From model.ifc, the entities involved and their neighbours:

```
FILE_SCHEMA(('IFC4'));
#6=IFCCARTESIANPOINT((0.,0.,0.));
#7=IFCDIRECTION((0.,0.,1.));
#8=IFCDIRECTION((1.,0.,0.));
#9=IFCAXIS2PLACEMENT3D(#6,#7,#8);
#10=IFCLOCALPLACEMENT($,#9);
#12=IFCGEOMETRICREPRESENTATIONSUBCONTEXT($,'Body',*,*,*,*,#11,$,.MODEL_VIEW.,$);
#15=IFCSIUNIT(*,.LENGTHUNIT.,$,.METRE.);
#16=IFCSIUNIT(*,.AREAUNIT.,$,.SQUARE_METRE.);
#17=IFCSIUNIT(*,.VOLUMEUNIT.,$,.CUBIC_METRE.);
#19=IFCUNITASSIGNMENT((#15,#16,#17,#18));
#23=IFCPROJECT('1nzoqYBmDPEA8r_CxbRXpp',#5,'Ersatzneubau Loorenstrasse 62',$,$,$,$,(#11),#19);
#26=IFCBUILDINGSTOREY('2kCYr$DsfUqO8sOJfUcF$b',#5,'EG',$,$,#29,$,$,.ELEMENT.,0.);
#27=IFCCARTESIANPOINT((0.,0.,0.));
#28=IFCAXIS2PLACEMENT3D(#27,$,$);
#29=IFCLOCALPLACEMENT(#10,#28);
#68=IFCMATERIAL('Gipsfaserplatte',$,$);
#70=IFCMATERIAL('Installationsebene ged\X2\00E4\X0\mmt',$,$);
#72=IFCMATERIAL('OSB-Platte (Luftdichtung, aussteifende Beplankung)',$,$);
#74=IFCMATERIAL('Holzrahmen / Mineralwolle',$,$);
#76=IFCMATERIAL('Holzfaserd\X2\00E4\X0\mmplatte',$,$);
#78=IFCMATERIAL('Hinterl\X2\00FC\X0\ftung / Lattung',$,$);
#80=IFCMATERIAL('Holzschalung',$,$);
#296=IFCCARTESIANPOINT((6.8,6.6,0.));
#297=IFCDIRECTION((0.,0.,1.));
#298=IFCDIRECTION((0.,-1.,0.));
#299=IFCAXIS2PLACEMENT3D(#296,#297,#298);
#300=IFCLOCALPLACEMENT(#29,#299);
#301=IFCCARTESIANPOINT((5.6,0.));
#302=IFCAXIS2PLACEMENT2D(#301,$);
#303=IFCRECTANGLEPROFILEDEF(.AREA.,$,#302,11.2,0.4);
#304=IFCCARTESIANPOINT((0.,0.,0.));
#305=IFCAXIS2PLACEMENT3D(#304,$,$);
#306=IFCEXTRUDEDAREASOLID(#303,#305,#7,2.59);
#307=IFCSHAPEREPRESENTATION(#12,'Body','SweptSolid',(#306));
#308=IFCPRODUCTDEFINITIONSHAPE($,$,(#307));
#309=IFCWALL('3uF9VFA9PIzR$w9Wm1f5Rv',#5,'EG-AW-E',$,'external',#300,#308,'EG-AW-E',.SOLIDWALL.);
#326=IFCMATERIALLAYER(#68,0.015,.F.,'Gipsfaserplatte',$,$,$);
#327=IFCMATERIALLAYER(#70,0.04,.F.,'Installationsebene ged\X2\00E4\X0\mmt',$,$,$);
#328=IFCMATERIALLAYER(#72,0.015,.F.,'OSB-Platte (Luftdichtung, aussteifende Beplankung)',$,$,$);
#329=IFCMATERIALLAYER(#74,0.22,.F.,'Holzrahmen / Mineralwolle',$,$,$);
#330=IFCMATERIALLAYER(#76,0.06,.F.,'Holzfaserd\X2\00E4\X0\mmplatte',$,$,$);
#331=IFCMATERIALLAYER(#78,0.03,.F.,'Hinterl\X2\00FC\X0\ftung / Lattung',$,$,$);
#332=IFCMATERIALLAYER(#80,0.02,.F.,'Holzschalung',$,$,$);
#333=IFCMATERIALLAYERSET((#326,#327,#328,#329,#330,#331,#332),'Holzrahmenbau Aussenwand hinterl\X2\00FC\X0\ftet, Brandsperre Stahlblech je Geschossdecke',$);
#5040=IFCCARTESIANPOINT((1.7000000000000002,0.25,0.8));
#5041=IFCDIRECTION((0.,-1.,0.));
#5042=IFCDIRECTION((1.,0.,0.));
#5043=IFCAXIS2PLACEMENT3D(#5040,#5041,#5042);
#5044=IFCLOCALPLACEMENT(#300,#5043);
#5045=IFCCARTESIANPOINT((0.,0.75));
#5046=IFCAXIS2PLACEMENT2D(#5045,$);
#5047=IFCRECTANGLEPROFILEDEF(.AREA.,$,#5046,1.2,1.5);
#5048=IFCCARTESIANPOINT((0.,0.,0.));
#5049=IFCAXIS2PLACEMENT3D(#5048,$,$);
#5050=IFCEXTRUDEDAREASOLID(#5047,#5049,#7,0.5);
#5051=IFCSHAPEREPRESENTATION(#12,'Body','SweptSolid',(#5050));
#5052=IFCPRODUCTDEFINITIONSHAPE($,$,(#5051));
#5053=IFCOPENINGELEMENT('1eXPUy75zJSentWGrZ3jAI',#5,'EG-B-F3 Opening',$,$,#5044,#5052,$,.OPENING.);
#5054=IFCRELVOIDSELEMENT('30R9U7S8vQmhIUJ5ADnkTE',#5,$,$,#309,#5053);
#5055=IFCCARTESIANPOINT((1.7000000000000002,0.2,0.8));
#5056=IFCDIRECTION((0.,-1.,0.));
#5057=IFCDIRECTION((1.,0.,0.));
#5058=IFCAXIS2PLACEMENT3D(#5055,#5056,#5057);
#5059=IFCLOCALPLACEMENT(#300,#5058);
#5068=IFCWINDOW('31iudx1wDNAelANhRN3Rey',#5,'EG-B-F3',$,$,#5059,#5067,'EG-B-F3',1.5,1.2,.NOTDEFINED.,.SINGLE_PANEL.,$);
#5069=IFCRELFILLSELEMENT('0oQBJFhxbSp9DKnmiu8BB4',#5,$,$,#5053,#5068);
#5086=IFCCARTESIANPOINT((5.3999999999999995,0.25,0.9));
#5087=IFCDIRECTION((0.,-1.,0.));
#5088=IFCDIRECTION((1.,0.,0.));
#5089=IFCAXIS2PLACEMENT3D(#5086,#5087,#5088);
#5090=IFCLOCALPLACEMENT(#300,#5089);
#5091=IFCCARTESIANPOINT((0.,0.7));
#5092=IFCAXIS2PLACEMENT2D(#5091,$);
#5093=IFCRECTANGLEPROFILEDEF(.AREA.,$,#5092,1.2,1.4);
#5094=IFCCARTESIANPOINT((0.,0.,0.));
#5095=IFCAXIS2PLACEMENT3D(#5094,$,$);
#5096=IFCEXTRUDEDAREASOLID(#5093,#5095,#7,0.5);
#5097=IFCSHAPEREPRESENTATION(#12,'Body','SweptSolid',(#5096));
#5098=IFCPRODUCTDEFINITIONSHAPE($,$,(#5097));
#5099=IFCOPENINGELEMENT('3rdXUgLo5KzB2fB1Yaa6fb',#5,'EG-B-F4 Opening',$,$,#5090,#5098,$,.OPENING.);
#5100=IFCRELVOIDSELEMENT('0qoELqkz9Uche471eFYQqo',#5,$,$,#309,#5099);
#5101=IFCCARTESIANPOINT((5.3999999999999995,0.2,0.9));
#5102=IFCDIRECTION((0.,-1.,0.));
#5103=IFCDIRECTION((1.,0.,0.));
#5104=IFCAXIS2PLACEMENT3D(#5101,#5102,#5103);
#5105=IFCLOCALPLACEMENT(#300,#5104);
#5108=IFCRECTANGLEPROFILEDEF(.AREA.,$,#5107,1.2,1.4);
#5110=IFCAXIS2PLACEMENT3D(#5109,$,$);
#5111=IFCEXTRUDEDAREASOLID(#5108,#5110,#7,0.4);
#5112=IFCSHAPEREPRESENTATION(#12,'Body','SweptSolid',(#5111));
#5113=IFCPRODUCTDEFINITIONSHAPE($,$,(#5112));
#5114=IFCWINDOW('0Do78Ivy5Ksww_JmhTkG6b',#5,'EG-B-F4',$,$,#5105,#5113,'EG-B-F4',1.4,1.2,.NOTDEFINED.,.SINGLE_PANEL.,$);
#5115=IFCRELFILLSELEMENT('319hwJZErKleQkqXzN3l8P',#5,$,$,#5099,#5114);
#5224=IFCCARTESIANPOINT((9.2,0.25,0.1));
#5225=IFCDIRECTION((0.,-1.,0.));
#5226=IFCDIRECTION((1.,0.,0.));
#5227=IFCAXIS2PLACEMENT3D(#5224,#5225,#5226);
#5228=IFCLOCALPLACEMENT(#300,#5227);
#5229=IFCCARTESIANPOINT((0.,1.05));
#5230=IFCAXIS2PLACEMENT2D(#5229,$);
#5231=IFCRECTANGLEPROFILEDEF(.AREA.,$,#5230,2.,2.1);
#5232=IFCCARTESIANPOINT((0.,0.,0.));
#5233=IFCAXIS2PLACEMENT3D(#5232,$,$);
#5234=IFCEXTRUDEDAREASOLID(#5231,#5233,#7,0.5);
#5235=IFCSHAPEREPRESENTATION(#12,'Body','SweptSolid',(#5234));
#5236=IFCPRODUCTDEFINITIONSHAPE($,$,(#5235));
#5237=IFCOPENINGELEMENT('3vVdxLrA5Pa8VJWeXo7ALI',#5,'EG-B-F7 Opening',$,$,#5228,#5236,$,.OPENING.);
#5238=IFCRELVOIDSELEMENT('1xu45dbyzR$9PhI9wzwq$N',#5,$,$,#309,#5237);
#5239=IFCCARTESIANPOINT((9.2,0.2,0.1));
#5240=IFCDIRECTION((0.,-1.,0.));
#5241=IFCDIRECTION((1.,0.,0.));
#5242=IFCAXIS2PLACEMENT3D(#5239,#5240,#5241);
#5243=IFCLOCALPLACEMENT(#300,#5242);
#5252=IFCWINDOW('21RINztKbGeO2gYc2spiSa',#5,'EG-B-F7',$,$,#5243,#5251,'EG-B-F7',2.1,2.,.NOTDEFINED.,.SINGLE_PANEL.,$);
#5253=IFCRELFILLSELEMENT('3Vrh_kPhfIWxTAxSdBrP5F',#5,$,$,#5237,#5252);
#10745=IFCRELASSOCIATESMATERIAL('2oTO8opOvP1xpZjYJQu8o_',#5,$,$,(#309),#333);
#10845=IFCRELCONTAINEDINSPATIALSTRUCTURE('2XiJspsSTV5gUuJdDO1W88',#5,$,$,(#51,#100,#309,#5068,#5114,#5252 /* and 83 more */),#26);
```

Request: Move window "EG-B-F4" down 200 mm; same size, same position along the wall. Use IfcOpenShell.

```python
import numpy as np
import ifcopenshell
import ifcopenshell.api.geometry
import ifcopenshell.util.placement
import ifcopenshell.util.unit

model = ifcopenshell.open("model.ifc")
unit_scale = ifcopenshell.util.unit.calculate_unit_scale(model)

window = model.by_guid("0Do78Ivy5Ksww_JmhTkG6b")
opening = window.FillsVoids[0].RelatingOpeningElement
dz = -0.2 / unit_scale

shift = np.array([0.0, 0.0, dz])
# The window is not placed relative to its opening, so move both.
for product in (opening, window):
    matrix = ifcopenshell.util.placement.get_local_placement(product.ObjectPlacement)
    matrix[:3, 3] += shift
    ifcopenshell.api.geometry.edit_object_placement(model, product=product, matrix=matrix, is_si=False)

print(f"moved by {dz * unit_scale:+.3f} m")

model.write("model-out.ifc")
```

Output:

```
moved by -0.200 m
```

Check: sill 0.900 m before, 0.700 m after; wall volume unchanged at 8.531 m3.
